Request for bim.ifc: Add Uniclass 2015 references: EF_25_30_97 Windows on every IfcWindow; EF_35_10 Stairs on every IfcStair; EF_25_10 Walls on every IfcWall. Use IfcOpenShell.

First a look at what the model holds.

```python
import ifcopenshell

model = ifcopenshell.open("bim.ifc")
print(model.schema)
print("classifications:", [c.Name for c in model.by_type("IfcClassification")])
for ifc_class in ("IfcDoor", "IfcRoof", "IfcStair", "IfcWall", "IfcWindow"):
    print(ifc_class, len(model.by_type(ifc_class)))
```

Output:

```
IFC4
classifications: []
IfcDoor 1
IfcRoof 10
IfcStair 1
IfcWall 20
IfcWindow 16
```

```python
import ifcopenshell
import ifcopenshell.api.classification

model = ifcopenshell.open("bim.ifc")

system = ifcopenshell.api.classification.add_classification(model, classification="Uniclass 2015")

codes = {
    "IfcWindow": ("EF_25_30_97", "Windows"),
    "IfcStair": ("EF_35_10", "Stairs"),
    "IfcWall": ("EF_25_10", "Walls"),
}
for ifc_class, (code, name) in codes.items():
    products = model.by_type(ifc_class)
    ifcopenshell.api.classification.add_reference(
        model, products=products, classification=system, identification=code, name=name
    )
    print(code, len(products))

model.write("bim_rev.ifc")
```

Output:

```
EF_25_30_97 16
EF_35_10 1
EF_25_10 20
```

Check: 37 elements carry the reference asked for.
